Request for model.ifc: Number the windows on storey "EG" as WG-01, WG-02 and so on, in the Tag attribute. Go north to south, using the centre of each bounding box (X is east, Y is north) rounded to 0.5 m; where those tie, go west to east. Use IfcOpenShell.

First a look at what the model holds.

```python
import ifcopenshell
import ifcopenshell.util.element
import ifcopenshell.util.placement

model = ifcopenshell.open("model.ifc")
print(model.schema)
storey = next(s for s in model.by_type("IfcBuildingStorey") if s.Name == "EG")
windows = [e for e in ifcopenshell.util.element.get_decomposition(storey) if e.is_a("IfcWindow")]
for e in sorted(windows, key=lambda e: e.id()):
    origin = ifcopenshell.util.placement.get_local_placement(e.ObjectPlacement)[:3, 3]
    print(e.id(), e.Tag, e.Name, origin.round(2) + 0.0, sep=" | ")
```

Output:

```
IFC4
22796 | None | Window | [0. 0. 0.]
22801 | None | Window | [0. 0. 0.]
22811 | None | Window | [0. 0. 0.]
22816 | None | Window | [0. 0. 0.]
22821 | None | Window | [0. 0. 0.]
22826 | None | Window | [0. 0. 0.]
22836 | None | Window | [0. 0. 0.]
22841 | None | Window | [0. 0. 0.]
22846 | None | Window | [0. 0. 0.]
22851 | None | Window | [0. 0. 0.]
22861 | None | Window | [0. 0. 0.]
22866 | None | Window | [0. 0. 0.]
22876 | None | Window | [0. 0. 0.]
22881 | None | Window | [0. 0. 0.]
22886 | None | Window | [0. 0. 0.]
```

```python
import ifcopenshell
import ifcopenshell.geom
import ifcopenshell.util.element
import ifcopenshell.util.shape

model = ifcopenshell.open("model.ifc")
settings = ifcopenshell.geom.settings()
settings.set("use-world-coords", True)


def centre(element):
    shape = ifcopenshell.geom.create_shape(settings, element)
    return ifcopenshell.util.shape.get_bbox_centroid(shape.geometry)


storey = next(s for s in model.by_type("IfcBuildingStorey") if s.Name == "EG")
windows = [e for e in ifcopenshell.util.element.get_decomposition(storey) if e.is_a("IfcWindow")]

# Insertion points can sit at a corner or the storey origin, so sort by the geometry (in metres).
centres = {e: centre(e) for e in windows}
windows.sort(key=lambda e: (-round(centres[e][1] / 0.5), centres[e][0]))

for i, e in enumerate(windows, start=1):
    number = f"WG-{i:02d}"
    e.Tag = number
    print(e.id(), number)

model.write("model-out.ifc")
```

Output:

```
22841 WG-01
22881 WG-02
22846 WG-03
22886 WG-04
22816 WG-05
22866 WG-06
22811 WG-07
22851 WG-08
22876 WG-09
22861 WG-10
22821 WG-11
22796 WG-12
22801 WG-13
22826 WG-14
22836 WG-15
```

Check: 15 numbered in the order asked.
